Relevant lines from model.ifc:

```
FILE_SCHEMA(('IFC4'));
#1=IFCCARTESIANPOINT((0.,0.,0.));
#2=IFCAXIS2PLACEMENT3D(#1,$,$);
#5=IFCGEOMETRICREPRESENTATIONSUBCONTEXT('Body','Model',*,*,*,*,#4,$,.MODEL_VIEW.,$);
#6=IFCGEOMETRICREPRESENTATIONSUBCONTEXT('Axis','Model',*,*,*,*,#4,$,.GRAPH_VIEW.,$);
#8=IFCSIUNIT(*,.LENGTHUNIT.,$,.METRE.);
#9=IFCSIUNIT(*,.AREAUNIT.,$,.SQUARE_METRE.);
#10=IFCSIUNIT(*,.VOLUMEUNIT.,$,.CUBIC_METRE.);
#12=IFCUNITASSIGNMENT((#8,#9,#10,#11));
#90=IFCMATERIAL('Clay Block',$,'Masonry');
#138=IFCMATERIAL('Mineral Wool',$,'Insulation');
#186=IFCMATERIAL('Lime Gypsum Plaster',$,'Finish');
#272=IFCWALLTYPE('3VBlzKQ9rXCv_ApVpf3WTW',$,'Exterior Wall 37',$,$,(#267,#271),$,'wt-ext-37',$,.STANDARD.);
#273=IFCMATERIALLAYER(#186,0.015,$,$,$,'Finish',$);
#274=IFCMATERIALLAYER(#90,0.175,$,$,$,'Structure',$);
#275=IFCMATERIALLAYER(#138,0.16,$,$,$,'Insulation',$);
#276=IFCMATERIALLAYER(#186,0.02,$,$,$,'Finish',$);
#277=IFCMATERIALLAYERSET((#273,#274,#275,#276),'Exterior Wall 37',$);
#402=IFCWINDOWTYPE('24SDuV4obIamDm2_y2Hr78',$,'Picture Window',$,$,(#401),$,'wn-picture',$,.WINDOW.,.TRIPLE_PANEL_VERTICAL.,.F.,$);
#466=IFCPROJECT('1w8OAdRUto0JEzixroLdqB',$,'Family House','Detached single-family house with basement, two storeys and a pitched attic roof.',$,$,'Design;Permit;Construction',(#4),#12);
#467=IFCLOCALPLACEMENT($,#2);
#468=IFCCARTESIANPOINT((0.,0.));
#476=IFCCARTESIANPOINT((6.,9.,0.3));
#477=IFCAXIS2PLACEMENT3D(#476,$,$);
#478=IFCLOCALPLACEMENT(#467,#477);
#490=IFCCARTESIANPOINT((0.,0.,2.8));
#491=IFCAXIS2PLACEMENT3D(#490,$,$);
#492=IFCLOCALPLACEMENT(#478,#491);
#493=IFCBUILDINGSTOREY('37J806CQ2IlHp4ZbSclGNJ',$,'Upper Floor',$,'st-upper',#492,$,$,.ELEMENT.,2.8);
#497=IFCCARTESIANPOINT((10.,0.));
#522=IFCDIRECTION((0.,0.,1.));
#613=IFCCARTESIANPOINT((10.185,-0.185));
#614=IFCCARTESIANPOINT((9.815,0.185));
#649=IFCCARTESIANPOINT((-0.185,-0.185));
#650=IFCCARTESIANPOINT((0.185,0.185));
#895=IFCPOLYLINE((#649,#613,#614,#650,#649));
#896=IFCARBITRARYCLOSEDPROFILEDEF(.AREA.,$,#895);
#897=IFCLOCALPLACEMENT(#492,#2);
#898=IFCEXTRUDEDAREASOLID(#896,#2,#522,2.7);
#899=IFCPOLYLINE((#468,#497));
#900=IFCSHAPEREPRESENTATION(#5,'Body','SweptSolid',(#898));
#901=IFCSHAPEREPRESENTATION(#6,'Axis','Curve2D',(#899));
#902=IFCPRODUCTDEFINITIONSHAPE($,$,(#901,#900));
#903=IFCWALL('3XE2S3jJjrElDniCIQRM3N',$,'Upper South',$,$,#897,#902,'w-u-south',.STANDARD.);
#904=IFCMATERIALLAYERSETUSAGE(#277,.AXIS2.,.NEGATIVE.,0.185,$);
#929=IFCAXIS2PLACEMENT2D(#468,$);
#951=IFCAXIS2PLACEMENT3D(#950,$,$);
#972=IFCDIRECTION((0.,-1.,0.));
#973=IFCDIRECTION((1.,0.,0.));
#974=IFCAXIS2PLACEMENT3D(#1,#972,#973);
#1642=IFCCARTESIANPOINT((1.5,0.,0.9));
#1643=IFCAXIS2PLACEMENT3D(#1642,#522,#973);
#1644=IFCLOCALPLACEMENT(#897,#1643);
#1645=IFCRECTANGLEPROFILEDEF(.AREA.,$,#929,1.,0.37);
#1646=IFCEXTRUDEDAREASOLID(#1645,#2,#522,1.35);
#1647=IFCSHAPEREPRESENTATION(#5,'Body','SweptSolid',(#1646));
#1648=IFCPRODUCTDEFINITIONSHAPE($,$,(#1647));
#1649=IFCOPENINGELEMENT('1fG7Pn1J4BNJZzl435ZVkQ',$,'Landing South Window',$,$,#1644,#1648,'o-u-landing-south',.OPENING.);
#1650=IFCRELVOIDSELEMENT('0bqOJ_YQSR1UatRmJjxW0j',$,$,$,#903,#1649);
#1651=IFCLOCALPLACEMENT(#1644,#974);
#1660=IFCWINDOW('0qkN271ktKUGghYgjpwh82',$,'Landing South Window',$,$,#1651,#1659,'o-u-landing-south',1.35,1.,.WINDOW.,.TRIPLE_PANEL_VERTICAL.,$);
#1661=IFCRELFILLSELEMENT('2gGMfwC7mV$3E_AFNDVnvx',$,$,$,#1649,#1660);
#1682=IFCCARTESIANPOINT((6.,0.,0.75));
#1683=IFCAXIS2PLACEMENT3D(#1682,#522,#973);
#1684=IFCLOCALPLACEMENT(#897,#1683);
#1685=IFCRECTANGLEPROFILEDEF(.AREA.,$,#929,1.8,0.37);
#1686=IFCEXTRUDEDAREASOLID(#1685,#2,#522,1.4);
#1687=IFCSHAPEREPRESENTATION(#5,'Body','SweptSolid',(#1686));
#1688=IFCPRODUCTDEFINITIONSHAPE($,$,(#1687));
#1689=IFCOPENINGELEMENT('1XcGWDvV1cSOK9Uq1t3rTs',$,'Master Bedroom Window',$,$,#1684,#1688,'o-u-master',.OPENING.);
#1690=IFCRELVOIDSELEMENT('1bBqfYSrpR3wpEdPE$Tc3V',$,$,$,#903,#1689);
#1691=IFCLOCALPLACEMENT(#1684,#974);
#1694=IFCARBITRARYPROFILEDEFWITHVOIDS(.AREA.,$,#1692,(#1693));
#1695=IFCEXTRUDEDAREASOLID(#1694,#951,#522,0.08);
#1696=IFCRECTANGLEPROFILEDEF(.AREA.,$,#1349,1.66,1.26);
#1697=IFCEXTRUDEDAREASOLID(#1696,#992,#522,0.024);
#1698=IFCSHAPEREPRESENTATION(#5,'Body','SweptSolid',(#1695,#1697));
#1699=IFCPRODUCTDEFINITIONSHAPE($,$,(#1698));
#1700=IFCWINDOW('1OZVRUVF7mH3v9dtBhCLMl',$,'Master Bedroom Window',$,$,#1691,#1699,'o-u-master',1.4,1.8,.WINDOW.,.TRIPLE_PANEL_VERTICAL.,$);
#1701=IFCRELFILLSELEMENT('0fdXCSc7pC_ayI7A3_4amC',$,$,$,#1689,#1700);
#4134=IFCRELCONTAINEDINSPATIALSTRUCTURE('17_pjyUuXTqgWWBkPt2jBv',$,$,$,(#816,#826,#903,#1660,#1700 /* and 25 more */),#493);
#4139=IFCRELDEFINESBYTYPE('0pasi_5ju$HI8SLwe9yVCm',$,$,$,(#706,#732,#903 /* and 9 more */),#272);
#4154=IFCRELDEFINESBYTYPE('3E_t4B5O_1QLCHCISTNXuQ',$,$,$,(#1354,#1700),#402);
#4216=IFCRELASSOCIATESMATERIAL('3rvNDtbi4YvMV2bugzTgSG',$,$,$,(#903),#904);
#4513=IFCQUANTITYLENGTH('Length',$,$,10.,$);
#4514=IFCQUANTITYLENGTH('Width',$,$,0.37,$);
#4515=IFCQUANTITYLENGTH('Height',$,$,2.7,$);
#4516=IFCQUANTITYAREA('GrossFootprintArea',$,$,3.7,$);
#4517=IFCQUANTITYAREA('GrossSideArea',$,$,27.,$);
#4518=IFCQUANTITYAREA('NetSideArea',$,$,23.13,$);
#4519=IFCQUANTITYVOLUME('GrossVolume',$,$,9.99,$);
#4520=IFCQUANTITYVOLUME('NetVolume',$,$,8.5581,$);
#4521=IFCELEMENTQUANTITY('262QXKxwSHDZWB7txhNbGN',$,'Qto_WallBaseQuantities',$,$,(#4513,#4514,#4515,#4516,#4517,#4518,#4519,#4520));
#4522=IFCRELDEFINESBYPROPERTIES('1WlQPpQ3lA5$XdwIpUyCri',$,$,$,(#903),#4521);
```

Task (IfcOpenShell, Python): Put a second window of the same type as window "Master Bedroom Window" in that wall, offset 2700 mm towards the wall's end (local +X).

```python
import ifcopenshell
import ifcopenshell.api.feature
import ifcopenshell.api.geometry
import ifcopenshell.api.pset
import ifcopenshell.api.root
import ifcopenshell.geom
import ifcopenshell.util.element
import ifcopenshell.util.placement
import ifcopenshell.util.shape
import ifcopenshell.util.unit

model = ifcopenshell.open("model.ifc")
unit_scale = ifcopenshell.util.unit.calculate_unit_scale(model)
area_scale = ifcopenshell.util.unit.calculate_unit_scale(model, "AREAUNIT")
volume_scale = ifcopenshell.util.unit.calculate_unit_scale(model, "VOLUMEUNIT")
settings = ifcopenshell.geom.settings()


def volume(element):
    """Net volume in cubic metres, openings subtracted."""
    shape = ifcopenshell.geom.create_shape(settings, element)
    return ifcopenshell.util.shape.get_volume(shape.geometry)


window = model.by_guid("1OZVRUVF7mH3v9dtBhCLMl")
opening = window.FillsVoids[0].RelatingOpeningElement
wall = opening.VoidsElements[0].RelatingBuildingElement
before = volume(wall)
shift = ifcopenshell.util.placement.get_local_placement(wall.ObjectPlacement)[:3, 0] * 2.7 / unit_scale

# copy_class copies the void relationship, type, container and properties, but no geometry.
new_opening = ifcopenshell.api.root.copy_class(model, product=opening)
new_opening.Representation = ifcopenshell.util.element.copy_deep(
    model, opening.Representation, exclude=["IfcGeometricRepresentationContext", "IfcRepresentationMap"]
)
new_opening.Tag = None
new_window = ifcopenshell.api.root.copy_class(model, product=window)
new_window.Representation = ifcopenshell.util.element.copy_deep(
    model, window.Representation, exclude=["IfcGeometricRepresentationContext", "IfcRepresentationMap"]
)
new_window.Tag = None
ifcopenshell.api.feature.add_filling(model, opening=new_opening, element=new_window)

for old, new in ((opening, new_opening), (window, new_window)):
    matrix = ifcopenshell.util.placement.get_local_placement(old.ObjectPlacement)
    matrix[:3, 3] += shift
    ifcopenshell.api.geometry.edit_object_placement(model, product=new, matrix=matrix, is_si=False)

after = volume(wall)
thickness = 0.37  # wall thickness in metres

# Update the wall's stored quantities.
qto = model.by_id(ifcopenshell.util.element.get_pset(wall, "Qto_WallBaseQuantities", should_inherit=False)["id"])
ifcopenshell.api.pset.edit_qto(model, qto=qto, properties={
    "NetSideArea": after / thickness / area_scale,
    "NetVolume": after / volume_scale,
})

print(f"wall volume {before:.3f} -> {after:.3f} m3")

model.write("model_edited.ifc")
```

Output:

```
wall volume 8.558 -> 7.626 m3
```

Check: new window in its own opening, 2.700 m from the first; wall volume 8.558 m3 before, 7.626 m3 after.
